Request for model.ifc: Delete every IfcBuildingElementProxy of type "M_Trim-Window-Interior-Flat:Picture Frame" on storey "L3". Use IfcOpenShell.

First a look at what the model holds.

```python
import ifcopenshell
import ifcopenshell.util.element

model = ifcopenshell.open("model.ifc")
print(model.schema)
storey = next(s for s in model.by_type("IfcBuildingStorey") if s.Name == "L3")
proxies = [e for e in ifcopenshell.util.element.get_decomposition(storey) if e.is_a("IfcBuildingElementProxy")]
seen = {}
for e in proxies:
    element_type = ifcopenshell.util.element.get_type(e)
    name = element_type.Name if element_type not in (None, e) else None
    seen[name] = seen.get(name, 0) + 1
for name, count in sorted(seen.items(), key=str):
    print(count, "x", name)
```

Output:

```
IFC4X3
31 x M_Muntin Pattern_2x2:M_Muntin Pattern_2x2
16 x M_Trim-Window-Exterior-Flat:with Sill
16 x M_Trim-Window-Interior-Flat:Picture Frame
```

```python
import ifcopenshell
import ifcopenshell.api.root
import ifcopenshell.util.element

model = ifcopenshell.open("model.ifc")

storey = next(s for s in model.by_type("IfcBuildingStorey") if s.Name == "L3")
proxies = [e for e in ifcopenshell.util.element.get_decomposition(storey) if e.is_a("IfcBuildingElementProxy")]
targets = [e for e in proxies if (t := ifcopenshell.util.element.get_type(e)) not in (None, e) and t.Name == "M_Trim-Window-Interior-Flat:Picture Frame"]

for e in targets:
    ifcopenshell.api.root.remove_product(model, product=e)
print(len(targets), "removed")

model.write("model-out.ifc")
```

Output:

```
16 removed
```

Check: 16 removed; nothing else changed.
